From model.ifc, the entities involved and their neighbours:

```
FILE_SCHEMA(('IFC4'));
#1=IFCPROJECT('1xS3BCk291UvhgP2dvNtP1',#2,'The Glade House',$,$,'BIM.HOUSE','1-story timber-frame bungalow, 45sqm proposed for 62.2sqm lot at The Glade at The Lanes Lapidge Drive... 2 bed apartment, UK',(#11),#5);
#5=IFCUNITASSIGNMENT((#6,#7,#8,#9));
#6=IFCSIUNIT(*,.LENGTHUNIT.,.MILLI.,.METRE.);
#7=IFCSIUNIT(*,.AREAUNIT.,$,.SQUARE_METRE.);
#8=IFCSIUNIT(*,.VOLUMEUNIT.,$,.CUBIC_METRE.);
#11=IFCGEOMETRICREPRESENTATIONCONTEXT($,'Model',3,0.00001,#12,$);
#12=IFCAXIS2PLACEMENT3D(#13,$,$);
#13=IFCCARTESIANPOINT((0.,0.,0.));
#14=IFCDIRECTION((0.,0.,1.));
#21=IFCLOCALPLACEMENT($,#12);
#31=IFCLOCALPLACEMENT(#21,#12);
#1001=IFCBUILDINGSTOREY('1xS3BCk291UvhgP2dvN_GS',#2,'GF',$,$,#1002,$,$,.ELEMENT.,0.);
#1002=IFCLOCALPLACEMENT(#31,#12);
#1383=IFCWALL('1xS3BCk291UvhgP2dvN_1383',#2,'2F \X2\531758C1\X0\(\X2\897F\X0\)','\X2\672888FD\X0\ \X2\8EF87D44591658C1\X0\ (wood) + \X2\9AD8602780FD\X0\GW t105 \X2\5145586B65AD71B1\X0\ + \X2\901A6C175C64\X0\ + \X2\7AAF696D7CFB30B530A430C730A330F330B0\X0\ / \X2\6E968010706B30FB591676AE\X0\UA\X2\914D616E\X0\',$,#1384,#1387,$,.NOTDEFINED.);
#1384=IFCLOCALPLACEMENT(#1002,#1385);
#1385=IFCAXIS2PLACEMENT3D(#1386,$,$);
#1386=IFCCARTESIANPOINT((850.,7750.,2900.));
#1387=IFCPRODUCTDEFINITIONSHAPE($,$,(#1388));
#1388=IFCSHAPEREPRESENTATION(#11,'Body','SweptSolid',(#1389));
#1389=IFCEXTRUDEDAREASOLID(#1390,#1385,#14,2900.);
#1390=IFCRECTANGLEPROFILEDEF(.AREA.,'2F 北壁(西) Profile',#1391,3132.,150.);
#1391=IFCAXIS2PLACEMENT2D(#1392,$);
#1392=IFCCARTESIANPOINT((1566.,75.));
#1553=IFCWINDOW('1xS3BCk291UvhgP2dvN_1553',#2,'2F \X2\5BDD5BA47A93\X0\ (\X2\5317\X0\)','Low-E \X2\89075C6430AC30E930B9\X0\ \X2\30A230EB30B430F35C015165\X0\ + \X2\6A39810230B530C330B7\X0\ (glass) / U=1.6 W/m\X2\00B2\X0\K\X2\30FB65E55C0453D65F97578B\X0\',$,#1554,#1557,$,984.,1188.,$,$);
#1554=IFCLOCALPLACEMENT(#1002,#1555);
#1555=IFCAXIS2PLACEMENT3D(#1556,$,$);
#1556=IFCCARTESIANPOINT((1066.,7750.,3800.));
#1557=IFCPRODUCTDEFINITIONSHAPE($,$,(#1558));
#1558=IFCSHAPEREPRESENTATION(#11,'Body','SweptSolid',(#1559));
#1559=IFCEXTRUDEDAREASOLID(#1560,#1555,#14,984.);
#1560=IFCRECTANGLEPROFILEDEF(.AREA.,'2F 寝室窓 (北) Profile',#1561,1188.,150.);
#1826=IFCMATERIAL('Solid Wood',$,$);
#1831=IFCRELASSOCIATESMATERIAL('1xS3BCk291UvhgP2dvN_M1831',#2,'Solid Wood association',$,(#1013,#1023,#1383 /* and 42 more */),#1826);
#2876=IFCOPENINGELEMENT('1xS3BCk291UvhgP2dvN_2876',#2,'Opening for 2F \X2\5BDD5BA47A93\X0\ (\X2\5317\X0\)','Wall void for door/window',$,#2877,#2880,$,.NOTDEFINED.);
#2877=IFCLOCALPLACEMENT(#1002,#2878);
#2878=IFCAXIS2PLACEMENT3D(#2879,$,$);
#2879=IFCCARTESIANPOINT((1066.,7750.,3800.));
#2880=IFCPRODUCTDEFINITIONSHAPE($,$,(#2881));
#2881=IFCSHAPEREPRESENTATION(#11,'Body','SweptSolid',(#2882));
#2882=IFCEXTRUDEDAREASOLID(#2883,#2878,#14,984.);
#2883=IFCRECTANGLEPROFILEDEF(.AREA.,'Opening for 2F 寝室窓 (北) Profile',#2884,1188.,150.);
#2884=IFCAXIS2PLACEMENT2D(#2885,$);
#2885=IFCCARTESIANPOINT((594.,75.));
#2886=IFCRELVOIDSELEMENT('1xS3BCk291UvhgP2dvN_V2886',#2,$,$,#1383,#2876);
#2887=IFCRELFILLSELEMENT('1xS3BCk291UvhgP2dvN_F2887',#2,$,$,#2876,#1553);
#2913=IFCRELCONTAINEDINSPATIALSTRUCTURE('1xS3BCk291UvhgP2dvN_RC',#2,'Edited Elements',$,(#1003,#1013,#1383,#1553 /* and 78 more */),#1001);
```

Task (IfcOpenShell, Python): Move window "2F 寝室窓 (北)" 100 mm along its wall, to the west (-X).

```python
import ifcopenshell
import ifcopenshell.api.geometry
import ifcopenshell.util.placement

model = ifcopenshell.open("model.ifc")

window = model.by_guid("1xS3BCk291UvhgP2dvN_1553")
opening = window.FillsVoids[0].RelatingOpeningElement
wall = opening.VoidsElements[0].RelatingBuildingElement

wall_matrix = ifcopenshell.util.placement.get_local_placement(wall.ObjectPlacement)
shift = wall_matrix[:3, 0] * -100.0
before = ifcopenshell.util.placement.get_local_placement(window.ObjectPlacement)[:3, 3].copy()

# The window is not placed relative to its opening, so move both.
for product in (opening, window):
    matrix = ifcopenshell.util.placement.get_local_placement(product.ObjectPlacement)
    matrix[:3, 3] += shift
    ifcopenshell.api.geometry.edit_object_placement(model, product=product, matrix=matrix, is_si=False)

after = ifcopenshell.util.placement.get_local_placement(window.ObjectPlacement)[:3, 3]
print("window moved by", (after - before).round(3) + 0.0)

model.write("model_v2.ifc")
```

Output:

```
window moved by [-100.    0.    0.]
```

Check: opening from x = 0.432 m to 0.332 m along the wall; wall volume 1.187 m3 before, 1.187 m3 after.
